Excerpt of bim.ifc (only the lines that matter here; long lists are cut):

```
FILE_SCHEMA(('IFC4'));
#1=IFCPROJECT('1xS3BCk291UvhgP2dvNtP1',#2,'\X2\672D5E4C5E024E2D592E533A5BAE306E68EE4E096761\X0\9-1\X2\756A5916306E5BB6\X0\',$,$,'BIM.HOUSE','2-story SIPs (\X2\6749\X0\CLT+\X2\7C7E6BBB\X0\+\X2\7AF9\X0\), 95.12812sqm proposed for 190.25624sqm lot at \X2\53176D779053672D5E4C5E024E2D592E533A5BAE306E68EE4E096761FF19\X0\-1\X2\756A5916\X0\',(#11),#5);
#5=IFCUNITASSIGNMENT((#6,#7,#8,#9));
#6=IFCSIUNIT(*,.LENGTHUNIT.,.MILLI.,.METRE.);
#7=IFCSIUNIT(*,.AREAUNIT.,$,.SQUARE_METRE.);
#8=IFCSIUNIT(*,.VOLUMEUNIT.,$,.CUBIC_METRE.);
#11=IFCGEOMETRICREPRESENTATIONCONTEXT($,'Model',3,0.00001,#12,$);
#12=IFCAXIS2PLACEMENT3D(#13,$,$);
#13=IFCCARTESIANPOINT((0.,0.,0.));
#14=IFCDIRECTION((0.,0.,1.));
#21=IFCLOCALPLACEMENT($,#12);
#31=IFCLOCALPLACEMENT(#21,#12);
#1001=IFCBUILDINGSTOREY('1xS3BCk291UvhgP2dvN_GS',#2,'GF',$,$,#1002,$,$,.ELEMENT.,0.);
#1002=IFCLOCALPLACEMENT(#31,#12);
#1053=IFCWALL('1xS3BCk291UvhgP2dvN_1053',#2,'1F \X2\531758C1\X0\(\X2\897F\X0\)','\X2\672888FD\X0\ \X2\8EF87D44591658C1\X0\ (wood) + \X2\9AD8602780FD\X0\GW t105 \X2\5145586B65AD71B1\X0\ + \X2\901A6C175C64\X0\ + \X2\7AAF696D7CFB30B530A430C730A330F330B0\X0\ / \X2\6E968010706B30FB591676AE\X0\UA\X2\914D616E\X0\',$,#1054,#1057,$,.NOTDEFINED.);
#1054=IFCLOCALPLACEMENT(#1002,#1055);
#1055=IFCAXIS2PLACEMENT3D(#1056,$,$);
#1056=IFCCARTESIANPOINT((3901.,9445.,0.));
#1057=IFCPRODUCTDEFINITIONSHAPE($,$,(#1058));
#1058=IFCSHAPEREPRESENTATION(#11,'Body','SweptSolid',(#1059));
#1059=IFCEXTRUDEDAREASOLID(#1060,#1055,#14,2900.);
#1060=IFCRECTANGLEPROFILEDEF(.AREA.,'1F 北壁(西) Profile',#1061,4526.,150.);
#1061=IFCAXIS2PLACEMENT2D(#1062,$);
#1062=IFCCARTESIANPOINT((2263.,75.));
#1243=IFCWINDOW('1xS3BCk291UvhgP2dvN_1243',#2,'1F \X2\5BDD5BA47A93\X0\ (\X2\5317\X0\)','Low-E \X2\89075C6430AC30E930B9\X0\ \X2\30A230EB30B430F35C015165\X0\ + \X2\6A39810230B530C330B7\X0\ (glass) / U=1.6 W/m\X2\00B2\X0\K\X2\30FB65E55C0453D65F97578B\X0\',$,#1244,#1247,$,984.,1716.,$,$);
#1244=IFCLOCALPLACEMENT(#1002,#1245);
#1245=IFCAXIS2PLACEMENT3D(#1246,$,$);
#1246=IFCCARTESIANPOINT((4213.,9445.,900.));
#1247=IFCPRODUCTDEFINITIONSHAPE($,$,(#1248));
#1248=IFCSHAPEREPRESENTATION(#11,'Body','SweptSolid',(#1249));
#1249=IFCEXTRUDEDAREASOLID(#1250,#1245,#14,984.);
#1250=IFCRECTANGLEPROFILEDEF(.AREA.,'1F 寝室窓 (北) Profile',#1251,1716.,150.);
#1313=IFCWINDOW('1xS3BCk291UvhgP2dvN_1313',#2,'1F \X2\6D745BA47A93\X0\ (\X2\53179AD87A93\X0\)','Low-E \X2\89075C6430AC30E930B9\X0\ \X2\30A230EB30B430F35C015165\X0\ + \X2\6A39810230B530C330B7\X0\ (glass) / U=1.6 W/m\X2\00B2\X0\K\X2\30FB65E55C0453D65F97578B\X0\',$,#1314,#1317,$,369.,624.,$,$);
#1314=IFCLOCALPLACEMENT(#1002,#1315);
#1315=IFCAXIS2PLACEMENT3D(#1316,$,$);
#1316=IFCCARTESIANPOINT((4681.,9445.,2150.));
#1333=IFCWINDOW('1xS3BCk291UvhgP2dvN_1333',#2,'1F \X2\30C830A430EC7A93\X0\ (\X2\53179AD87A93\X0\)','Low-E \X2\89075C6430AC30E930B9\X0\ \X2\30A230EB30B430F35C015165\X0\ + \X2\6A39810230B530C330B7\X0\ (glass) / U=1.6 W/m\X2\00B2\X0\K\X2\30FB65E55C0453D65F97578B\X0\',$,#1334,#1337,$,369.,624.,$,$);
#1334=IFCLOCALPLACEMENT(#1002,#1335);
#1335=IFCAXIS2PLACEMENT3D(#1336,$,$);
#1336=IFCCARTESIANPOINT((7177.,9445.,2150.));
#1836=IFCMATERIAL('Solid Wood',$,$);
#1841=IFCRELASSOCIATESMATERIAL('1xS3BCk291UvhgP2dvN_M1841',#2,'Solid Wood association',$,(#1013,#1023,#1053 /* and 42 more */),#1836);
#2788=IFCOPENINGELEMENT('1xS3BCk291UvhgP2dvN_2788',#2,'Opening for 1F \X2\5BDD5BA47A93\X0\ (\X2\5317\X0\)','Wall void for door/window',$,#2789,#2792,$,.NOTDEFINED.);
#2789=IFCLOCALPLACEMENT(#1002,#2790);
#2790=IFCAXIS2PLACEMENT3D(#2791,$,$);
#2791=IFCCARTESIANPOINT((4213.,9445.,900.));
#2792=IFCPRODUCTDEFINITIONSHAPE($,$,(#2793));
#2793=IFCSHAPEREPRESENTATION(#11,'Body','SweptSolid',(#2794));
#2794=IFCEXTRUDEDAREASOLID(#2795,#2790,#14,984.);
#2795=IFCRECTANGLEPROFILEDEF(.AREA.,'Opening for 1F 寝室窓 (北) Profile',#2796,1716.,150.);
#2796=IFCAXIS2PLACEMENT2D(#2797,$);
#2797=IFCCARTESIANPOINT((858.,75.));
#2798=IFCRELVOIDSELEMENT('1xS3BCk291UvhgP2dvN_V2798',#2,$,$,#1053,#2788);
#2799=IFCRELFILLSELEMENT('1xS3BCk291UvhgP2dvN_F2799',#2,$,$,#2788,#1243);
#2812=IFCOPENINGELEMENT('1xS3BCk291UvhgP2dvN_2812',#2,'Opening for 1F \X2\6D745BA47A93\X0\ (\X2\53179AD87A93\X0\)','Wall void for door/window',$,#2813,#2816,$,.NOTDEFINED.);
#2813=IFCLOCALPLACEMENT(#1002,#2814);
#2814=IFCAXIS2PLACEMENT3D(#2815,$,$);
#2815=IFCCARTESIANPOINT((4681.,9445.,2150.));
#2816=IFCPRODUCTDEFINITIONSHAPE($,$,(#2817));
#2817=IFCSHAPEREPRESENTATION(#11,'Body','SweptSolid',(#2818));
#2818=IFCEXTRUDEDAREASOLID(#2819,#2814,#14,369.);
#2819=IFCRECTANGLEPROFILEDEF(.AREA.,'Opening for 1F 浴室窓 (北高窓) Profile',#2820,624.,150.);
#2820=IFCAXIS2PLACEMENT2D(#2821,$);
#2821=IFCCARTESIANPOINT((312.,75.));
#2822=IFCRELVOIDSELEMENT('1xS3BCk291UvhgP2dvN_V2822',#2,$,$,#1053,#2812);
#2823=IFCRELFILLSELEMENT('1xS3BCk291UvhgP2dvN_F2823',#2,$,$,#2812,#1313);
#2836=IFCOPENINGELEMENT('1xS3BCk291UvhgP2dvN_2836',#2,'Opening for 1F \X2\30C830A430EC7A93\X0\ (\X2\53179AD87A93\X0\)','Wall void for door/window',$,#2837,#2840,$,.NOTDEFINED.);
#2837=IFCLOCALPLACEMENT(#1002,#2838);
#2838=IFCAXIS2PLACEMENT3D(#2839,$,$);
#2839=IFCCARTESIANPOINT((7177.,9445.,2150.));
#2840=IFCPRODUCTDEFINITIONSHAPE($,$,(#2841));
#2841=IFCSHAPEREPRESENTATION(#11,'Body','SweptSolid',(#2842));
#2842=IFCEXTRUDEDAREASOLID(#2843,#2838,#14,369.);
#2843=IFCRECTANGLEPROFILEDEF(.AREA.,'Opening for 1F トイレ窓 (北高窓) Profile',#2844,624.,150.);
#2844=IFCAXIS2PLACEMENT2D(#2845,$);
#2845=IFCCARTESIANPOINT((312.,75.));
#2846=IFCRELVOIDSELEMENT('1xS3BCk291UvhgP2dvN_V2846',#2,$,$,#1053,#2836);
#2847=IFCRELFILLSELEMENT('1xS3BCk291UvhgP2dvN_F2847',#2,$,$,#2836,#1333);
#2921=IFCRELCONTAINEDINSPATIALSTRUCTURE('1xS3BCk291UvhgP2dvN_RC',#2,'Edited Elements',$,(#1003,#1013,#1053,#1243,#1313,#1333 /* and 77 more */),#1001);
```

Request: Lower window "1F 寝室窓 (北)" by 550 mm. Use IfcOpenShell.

```python
import numpy as np
import ifcopenshell
import ifcopenshell.api.geometry
import ifcopenshell.util.placement
import ifcopenshell.util.unit

model = ifcopenshell.open("bim.ifc")
unit_scale = ifcopenshell.util.unit.calculate_unit_scale(model)

window = model.by_id(1243)
opening = window.FillsVoids[0].RelatingOpeningElement
dz = -0.55 / unit_scale

shift = np.array([0.0, 0.0, dz])
# The window is not placed relative to its opening, so move both.
for product in (opening, window):
    matrix = ifcopenshell.util.placement.get_local_placement(product.ObjectPlacement)
    matrix[:3, 3] += shift
    ifcopenshell.api.geometry.edit_object_placement(model, product=product, matrix=matrix, is_si=False)

print(f"moved by {dz * unit_scale:+.3f} m")

model.write("bim_edited.ifc")
```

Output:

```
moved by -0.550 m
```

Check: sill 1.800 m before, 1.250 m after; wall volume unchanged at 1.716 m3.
